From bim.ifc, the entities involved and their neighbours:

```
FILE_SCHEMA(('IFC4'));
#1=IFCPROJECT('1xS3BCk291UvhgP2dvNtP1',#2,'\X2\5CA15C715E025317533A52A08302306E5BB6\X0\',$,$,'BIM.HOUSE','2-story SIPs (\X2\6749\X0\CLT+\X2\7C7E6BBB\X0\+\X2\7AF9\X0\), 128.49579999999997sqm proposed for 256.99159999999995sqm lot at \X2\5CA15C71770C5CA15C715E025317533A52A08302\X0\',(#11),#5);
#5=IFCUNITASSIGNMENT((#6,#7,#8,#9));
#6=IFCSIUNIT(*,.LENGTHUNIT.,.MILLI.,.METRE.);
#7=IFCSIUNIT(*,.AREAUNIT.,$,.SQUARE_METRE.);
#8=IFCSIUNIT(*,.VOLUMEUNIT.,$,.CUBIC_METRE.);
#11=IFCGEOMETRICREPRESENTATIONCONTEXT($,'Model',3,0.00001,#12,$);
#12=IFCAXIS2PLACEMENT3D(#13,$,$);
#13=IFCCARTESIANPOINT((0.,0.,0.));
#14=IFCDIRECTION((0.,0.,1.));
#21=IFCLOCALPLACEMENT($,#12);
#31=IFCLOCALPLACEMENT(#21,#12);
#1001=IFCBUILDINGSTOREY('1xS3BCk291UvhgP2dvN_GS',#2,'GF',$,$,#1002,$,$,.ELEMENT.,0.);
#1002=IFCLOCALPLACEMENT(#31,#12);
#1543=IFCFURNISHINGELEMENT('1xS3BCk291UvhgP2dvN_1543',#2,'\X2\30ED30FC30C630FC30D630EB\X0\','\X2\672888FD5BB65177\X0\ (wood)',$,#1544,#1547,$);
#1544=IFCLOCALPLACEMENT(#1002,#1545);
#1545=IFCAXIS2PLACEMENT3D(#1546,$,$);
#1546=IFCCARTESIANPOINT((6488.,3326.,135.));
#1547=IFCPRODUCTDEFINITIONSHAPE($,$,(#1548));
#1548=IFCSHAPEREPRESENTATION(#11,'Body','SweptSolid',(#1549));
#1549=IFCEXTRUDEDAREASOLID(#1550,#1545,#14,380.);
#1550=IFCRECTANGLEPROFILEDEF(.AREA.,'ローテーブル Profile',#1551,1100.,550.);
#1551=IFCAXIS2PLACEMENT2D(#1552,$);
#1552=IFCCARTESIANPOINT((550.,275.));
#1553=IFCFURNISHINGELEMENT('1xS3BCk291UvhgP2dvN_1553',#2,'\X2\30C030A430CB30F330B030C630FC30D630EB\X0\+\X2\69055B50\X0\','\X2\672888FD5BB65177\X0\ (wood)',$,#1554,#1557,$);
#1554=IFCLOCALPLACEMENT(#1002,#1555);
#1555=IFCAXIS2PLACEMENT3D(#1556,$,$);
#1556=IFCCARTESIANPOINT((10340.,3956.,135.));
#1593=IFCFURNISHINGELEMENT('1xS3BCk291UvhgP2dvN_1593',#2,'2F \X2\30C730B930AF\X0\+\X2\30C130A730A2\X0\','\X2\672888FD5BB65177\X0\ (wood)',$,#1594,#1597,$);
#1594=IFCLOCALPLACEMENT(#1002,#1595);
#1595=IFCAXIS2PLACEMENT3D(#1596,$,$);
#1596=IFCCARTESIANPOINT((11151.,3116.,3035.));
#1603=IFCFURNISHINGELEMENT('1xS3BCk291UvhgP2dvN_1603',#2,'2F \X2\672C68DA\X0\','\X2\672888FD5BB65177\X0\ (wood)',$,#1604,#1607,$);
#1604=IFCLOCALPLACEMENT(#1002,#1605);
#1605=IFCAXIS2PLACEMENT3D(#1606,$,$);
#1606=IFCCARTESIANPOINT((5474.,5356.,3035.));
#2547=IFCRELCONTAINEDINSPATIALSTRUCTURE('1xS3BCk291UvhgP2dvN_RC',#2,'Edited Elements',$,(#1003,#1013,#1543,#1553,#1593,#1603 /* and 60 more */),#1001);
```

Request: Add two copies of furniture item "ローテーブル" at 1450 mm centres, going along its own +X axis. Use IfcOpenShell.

```python
import ifcopenshell
import ifcopenshell.api.geometry
import ifcopenshell.api.root
import ifcopenshell.util.element
import ifcopenshell.util.placement
import ifcopenshell.util.unit

model = ifcopenshell.open("bim.ifc")
unit_scale = ifcopenshell.util.unit.calculate_unit_scale(model)


def reuse_history(source, copy):
    """copy_class also copies each property set's owner history, people and application; keep the originals."""
    for rel in copy.IsDefinedBy:
        if rel.is_a("IfcRelDefinesByProperties") and (history := rel.RelatingPropertyDefinition.OwnerHistory):
            rel.RelatingPropertyDefinition.OwnerHistory = source.OwnerHistory
            ifcopenshell.util.element.remove_deep2(model, history)


source = model.by_guid("1xS3BCk291UvhgP2dvN_1543")
base = ifcopenshell.util.placement.get_local_placement(source.ObjectPlacement)
step = base[:3, 0] * 1.45 / unit_scale

for i in range(1, 3):
    copy = ifcopenshell.api.root.copy_class(model, product=source)
    copy.Representation = ifcopenshell.util.element.copy_deep(
        model, source.Representation, exclude=["IfcGeometricRepresentationContext", "IfcRepresentationMap"]
    )
    reuse_history(source, copy)
    matrix = base.copy()
    matrix[:3, 3] += i * step
    print("added at", matrix[:3, 3].round(3) + 0.0)
    ifcopenshell.api.geometry.edit_object_placement(model, product=copy, matrix=matrix, is_si=False)

model.write("bim_rev.ifc")
```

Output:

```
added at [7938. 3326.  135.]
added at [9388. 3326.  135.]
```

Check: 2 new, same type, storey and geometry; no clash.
